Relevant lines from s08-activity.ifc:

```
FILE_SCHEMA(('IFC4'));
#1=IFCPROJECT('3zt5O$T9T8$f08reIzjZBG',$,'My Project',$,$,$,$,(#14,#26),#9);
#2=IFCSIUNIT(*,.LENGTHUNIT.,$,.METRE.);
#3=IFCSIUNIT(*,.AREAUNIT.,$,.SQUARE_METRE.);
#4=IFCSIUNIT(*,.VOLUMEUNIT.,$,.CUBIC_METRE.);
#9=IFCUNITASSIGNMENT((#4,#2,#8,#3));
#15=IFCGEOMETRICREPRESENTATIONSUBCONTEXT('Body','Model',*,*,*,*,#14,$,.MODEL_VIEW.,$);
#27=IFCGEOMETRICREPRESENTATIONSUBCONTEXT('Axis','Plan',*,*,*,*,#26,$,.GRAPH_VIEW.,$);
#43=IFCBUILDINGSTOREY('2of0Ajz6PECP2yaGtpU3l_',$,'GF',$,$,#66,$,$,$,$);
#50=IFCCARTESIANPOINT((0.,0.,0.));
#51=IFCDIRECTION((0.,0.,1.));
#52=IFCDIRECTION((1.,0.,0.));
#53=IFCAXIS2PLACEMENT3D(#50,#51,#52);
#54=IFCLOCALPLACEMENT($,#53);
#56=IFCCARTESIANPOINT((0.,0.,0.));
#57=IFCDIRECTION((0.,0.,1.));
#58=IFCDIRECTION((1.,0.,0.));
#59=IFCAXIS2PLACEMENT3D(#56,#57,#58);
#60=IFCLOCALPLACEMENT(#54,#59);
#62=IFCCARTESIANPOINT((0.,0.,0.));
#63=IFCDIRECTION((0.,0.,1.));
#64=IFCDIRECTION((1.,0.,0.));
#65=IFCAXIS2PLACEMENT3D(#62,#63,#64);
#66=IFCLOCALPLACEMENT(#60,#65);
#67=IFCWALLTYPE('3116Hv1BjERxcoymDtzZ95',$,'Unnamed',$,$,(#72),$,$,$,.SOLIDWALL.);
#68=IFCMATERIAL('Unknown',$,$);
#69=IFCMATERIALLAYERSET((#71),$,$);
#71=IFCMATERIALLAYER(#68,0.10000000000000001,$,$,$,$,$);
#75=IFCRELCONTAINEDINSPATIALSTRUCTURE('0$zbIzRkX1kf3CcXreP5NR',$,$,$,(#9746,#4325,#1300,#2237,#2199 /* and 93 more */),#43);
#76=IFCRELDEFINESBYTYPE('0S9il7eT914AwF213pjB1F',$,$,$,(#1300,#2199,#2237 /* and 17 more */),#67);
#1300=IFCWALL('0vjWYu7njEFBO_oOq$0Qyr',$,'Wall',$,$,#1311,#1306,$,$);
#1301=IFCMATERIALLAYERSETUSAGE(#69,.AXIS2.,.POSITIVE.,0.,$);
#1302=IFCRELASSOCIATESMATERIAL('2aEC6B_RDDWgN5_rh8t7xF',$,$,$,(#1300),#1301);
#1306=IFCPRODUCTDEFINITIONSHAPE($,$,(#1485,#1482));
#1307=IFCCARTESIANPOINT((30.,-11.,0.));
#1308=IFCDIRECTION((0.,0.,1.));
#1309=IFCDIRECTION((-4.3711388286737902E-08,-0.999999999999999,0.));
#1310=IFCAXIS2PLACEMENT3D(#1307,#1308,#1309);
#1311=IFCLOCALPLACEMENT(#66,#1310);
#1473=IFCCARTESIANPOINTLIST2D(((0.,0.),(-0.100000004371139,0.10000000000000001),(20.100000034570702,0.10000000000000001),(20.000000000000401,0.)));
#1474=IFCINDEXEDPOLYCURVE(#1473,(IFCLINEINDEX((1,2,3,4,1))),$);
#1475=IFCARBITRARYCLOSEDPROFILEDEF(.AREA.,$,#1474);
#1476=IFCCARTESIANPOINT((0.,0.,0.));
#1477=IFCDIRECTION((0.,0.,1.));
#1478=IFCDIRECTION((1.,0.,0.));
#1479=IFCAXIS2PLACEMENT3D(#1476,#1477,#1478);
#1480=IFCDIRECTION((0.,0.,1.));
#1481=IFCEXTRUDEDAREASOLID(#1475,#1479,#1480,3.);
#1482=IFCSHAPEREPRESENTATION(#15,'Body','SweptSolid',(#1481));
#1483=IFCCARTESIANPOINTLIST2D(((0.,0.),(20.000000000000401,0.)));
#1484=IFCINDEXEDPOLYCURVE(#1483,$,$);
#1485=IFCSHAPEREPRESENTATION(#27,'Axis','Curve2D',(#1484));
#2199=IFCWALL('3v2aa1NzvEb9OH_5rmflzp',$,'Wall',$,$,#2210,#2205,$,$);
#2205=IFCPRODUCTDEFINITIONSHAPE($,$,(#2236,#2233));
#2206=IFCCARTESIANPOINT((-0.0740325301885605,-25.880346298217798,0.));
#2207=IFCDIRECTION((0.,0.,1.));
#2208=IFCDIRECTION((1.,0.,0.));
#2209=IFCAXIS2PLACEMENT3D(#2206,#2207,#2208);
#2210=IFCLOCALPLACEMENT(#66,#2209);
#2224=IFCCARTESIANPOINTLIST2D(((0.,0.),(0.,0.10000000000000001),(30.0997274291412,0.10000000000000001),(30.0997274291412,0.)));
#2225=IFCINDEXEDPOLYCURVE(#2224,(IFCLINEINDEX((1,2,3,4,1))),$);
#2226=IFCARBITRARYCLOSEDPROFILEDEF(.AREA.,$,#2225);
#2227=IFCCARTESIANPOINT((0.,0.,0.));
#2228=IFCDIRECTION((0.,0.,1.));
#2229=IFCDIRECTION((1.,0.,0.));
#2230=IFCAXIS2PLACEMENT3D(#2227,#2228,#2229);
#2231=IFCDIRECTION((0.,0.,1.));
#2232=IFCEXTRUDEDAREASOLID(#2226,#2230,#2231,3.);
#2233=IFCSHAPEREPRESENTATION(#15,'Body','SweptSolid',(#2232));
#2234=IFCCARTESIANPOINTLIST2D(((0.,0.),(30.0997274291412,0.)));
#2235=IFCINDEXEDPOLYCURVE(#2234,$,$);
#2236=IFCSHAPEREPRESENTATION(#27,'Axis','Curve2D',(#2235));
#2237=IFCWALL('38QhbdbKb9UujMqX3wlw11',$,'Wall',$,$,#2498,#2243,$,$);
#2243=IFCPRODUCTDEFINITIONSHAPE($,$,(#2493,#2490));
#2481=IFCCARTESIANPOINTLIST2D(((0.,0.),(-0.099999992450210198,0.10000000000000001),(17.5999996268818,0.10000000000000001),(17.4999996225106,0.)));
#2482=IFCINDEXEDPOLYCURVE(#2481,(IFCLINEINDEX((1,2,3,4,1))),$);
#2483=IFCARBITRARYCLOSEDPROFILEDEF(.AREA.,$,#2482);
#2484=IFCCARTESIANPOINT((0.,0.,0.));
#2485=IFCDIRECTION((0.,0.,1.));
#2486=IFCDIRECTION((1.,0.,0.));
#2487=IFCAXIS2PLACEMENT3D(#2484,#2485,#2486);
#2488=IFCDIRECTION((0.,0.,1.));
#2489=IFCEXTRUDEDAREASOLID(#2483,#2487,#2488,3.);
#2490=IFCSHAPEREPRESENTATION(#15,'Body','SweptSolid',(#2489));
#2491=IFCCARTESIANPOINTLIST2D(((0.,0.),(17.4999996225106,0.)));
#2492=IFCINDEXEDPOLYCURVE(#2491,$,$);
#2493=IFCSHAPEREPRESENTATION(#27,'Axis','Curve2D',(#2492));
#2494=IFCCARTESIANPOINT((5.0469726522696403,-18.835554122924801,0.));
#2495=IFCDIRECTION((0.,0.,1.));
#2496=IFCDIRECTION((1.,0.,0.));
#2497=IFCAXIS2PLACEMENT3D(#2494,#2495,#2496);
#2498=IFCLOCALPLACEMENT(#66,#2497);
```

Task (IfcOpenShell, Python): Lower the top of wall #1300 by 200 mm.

```python
import ifcopenshell
import ifcopenshell.geom
import ifcopenshell.util.representation
import ifcopenshell.util.shape
import ifcopenshell.util.unit

model = ifcopenshell.open("s08-activity.ifc")
unit_scale = ifcopenshell.util.unit.calculate_unit_scale(model)
settings = ifcopenshell.geom.settings()


def volume(element):
    """Net volume in cubic metres, openings subtracted."""
    shape = ifcopenshell.geom.create_shape(settings, element)
    return ifcopenshell.util.shape.get_volume(shape.geometry)


wall = model.by_id(1300)
before = volume(wall)

body = ifcopenshell.util.representation.get_representation(wall, "Model", "Body")
solid = body.Items[0]
old_height = solid.Depth
solid.Depth -= 0.2 / unit_scale
after = volume(wall)

print(f"height {old_height:g} -> {solid.Depth:g}, volume {before:.3f} -> {after:.3f} m3")

model.write("s08-activity_v2.ifc")
```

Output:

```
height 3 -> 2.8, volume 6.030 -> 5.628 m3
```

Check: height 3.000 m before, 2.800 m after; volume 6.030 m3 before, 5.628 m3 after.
